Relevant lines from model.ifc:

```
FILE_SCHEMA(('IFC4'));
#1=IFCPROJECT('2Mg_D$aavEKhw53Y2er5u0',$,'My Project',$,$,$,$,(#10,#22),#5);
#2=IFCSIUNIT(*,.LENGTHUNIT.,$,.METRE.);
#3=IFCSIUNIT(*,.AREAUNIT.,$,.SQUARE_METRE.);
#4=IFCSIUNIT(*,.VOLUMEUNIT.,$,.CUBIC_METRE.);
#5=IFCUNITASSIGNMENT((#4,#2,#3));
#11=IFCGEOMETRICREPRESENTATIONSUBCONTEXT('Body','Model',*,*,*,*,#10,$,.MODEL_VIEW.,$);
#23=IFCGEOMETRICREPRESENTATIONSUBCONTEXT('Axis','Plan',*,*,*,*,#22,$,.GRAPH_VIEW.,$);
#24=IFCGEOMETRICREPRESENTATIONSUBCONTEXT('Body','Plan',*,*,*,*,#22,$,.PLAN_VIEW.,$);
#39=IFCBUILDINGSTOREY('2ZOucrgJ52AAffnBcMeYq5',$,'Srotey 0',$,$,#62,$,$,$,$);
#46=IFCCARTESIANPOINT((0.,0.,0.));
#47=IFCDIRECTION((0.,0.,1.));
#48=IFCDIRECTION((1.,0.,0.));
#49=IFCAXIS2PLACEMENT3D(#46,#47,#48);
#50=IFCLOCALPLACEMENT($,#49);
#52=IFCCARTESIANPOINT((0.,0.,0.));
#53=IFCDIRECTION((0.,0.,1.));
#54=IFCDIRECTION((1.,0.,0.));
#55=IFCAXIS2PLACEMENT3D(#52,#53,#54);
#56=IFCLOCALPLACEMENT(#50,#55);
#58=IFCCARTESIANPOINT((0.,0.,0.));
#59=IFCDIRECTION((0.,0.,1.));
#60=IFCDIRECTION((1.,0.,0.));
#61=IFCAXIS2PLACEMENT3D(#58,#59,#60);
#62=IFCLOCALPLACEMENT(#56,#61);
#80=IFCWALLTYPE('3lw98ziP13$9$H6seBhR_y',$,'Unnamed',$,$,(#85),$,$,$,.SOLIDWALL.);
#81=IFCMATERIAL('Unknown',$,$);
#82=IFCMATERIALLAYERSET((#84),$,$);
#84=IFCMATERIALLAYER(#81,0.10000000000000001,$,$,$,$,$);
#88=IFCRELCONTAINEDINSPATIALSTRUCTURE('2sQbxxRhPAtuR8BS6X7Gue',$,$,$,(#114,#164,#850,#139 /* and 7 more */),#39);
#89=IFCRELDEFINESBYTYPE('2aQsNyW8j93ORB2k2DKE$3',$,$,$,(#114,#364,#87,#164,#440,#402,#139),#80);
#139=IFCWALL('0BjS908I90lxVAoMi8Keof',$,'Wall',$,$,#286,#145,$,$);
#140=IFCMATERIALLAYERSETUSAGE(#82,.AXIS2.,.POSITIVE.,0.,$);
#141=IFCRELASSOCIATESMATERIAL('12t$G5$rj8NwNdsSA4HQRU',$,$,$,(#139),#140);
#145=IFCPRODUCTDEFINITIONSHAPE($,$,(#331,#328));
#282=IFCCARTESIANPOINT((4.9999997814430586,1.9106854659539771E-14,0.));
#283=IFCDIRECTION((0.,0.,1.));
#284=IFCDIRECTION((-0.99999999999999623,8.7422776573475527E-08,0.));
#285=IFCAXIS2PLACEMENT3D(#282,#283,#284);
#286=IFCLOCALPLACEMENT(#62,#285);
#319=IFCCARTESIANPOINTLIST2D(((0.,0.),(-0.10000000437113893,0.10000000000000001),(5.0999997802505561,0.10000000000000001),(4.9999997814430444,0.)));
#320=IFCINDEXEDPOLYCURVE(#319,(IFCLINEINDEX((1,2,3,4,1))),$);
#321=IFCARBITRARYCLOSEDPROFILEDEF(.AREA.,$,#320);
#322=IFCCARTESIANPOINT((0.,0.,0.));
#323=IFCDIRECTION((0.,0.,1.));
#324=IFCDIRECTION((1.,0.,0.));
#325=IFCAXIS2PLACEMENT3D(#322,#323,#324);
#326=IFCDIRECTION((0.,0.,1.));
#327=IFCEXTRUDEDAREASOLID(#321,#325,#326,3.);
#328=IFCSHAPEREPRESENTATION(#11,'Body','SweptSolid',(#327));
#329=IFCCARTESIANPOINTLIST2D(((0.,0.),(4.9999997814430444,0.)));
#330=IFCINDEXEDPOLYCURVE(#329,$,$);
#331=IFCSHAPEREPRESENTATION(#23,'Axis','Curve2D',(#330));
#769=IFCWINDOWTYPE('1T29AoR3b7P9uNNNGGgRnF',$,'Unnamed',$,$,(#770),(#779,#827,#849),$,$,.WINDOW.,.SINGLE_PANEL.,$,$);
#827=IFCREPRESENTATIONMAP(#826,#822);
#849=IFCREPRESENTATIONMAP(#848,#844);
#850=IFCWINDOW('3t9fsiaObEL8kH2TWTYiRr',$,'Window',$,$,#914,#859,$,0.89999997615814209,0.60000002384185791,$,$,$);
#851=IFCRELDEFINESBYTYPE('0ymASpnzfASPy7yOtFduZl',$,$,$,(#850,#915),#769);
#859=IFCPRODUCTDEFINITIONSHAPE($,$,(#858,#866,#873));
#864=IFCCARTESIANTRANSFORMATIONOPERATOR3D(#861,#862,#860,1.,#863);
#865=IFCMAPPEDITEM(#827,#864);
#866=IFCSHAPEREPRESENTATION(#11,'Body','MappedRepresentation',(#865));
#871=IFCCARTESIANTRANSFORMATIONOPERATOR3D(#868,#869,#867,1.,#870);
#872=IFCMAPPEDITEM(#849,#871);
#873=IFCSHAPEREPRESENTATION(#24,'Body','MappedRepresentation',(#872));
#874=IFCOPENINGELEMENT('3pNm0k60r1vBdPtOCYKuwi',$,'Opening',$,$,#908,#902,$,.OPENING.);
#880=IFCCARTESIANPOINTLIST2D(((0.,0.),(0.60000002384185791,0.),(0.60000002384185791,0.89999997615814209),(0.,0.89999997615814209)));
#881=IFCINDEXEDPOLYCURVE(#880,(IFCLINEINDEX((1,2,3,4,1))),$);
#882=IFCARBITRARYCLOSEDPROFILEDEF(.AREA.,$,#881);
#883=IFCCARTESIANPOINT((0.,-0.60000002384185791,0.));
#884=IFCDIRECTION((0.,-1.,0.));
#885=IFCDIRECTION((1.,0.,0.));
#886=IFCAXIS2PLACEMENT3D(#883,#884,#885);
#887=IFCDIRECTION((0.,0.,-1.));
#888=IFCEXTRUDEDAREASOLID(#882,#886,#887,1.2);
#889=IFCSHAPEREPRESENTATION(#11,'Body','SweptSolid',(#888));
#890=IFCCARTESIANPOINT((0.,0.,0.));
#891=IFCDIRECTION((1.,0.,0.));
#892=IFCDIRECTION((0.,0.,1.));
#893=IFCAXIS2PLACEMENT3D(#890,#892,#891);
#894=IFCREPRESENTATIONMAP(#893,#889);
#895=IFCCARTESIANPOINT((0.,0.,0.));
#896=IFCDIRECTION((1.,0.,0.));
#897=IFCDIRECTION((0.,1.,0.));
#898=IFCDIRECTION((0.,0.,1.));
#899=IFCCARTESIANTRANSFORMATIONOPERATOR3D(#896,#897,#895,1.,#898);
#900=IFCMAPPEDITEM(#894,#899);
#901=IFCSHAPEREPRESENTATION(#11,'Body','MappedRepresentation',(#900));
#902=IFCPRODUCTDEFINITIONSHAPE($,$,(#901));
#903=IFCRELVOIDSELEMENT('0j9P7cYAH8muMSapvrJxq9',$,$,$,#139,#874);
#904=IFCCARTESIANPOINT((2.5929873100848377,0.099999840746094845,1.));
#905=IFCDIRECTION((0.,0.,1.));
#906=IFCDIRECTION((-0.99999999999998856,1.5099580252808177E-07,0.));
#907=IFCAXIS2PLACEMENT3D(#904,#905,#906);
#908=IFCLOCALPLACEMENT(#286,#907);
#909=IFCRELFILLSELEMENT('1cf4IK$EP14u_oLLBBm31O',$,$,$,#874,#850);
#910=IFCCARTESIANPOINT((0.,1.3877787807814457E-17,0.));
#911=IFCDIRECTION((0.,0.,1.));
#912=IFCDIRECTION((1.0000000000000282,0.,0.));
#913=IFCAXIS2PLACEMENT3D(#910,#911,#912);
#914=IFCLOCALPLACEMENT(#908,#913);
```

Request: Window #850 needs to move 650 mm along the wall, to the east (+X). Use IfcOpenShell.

```python
import ifcopenshell
import ifcopenshell.api.geometry
import ifcopenshell.util.placement
import ifcopenshell.util.unit

model = ifcopenshell.open("model.ifc")
unit_scale = ifcopenshell.util.unit.calculate_unit_scale(model)

window = model.by_guid("3t9fsiaObEL8kH2TWTYiRr")
opening = window.FillsVoids[0].RelatingOpeningElement
wall = opening.VoidsElements[0].RelatingBuildingElement

wall_matrix = ifcopenshell.util.placement.get_local_placement(wall.ObjectPlacement)
shift = wall_matrix[:3, 0] * -0.65 / unit_scale
before = ifcopenshell.util.placement.get_local_placement(window.ObjectPlacement)[:3, 3].copy()

# The window is placed relative to its opening, so it follows when the opening moves.
matrix = ifcopenshell.util.placement.get_local_placement(opening.ObjectPlacement)
matrix[:3, 3] += shift
ifcopenshell.api.geometry.edit_object_placement(
    model, product=opening, matrix=matrix, is_si=False, should_transform_children=True
)

after = ifcopenshell.util.placement.get_local_placement(window.ObjectPlacement)[:3, 3]
print("window moved by", (after - before).round(3) + 0.0)

model.write("model_updated.ifc")
```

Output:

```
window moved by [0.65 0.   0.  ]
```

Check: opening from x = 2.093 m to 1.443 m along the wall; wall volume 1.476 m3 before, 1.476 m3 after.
